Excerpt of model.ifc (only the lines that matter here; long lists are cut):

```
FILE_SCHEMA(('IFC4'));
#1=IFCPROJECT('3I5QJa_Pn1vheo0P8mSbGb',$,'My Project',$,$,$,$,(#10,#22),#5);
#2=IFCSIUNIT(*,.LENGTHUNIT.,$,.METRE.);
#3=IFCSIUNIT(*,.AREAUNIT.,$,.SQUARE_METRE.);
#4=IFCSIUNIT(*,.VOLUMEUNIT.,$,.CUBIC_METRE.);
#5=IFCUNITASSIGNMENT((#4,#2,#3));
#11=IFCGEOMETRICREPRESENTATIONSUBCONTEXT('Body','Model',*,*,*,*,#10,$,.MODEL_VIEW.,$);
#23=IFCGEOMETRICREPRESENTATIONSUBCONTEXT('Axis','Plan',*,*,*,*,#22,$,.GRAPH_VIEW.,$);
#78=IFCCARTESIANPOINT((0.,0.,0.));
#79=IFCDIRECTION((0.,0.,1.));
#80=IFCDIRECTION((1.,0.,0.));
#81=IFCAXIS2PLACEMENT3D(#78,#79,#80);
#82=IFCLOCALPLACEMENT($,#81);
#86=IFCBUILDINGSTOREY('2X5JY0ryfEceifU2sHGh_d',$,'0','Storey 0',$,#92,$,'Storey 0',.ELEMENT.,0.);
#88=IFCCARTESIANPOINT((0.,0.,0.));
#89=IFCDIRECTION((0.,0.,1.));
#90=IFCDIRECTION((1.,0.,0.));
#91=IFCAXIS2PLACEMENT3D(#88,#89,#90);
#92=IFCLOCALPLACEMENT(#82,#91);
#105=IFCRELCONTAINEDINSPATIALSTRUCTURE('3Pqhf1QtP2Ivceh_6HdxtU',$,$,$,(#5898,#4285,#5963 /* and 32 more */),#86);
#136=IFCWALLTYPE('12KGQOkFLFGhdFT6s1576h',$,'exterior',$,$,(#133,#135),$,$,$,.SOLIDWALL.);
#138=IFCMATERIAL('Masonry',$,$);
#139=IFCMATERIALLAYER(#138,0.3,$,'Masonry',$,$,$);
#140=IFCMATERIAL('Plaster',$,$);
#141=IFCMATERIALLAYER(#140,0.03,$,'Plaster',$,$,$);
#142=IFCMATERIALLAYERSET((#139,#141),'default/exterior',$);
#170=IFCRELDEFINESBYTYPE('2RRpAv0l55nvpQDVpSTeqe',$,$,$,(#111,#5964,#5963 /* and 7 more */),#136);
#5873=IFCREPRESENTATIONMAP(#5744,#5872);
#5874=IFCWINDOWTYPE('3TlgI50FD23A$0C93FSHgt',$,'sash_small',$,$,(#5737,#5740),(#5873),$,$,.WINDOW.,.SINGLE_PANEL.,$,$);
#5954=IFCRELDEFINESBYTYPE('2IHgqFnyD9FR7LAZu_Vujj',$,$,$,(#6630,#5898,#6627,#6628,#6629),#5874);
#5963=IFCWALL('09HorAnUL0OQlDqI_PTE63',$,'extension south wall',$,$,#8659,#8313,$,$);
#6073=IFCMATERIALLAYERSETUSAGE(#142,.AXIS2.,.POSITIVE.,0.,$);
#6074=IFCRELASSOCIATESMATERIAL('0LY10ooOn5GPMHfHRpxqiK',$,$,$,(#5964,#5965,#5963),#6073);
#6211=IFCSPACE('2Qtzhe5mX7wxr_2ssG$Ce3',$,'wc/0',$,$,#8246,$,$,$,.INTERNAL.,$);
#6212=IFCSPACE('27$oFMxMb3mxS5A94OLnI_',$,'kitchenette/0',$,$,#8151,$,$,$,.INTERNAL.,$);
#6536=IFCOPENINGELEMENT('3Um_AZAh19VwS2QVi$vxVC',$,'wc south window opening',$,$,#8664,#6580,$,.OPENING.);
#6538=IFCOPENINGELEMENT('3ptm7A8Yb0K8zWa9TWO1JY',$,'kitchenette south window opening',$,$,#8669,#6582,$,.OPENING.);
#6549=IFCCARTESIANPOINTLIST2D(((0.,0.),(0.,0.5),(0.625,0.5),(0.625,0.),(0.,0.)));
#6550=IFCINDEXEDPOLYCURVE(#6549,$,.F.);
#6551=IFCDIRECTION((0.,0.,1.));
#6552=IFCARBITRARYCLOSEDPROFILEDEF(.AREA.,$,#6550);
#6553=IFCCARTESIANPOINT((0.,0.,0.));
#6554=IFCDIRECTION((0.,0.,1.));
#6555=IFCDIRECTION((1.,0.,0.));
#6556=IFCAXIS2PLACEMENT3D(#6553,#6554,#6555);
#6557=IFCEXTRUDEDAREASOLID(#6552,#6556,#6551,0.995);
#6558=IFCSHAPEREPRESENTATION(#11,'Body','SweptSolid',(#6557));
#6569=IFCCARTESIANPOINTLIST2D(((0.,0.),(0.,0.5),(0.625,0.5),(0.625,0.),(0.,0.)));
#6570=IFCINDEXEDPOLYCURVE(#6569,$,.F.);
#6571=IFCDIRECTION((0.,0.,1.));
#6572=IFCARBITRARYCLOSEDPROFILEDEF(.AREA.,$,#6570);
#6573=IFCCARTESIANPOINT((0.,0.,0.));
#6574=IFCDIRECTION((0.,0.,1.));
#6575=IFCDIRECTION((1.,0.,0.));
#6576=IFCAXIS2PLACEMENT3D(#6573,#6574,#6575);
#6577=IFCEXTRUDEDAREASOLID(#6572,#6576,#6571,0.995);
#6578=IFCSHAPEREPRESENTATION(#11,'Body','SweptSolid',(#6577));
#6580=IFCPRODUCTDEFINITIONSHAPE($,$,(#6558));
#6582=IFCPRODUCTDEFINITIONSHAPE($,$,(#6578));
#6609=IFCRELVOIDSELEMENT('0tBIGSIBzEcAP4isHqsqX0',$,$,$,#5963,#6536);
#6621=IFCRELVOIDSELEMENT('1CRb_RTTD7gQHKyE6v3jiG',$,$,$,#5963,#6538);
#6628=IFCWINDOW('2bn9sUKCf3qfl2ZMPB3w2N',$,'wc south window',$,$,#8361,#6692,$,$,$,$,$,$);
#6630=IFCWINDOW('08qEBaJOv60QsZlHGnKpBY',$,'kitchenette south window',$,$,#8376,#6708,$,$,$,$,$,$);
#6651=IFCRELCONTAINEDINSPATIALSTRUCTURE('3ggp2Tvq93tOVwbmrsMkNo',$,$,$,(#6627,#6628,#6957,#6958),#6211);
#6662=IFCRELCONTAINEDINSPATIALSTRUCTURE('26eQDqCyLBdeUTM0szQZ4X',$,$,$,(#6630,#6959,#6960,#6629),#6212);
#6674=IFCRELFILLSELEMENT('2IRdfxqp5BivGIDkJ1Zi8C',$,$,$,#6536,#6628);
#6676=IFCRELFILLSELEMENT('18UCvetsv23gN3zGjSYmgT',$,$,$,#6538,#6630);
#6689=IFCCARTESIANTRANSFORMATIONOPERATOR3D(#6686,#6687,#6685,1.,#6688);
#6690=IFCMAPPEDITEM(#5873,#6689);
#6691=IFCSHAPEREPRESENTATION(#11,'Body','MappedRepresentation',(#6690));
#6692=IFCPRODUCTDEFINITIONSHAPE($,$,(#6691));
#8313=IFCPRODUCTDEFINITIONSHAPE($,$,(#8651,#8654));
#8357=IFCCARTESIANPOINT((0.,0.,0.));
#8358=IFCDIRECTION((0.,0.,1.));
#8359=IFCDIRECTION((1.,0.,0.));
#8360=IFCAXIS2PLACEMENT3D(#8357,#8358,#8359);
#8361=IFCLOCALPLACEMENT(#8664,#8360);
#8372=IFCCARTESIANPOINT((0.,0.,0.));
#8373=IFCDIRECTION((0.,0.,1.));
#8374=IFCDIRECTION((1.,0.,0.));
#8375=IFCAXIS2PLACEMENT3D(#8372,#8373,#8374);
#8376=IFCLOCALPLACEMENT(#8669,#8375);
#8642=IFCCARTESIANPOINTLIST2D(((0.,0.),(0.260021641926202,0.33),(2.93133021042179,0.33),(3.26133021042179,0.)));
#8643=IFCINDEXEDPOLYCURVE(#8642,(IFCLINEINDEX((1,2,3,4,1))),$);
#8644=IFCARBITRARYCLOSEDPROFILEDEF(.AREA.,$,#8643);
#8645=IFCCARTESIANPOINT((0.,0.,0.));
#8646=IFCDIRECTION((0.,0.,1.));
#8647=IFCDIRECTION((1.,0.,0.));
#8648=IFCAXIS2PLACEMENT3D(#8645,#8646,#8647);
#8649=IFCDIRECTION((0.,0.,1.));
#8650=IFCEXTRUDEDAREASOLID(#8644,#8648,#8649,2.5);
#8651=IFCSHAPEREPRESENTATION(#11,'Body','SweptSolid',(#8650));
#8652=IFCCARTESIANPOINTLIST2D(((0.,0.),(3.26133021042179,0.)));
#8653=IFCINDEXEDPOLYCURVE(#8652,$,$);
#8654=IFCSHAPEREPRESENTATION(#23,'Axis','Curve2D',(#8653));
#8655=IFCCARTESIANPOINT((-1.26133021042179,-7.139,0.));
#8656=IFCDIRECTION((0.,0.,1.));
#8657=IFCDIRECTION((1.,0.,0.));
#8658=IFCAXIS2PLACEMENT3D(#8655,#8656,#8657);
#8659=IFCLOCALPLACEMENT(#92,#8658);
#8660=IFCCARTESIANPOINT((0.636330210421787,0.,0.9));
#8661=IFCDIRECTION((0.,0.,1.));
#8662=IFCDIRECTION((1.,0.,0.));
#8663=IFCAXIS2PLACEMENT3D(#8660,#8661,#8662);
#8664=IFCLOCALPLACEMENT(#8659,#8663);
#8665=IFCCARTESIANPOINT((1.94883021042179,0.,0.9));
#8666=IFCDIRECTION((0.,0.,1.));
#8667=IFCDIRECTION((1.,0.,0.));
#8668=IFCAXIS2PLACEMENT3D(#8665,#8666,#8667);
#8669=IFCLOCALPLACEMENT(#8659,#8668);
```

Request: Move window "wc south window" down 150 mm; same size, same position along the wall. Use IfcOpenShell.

```python
import numpy as np
import ifcopenshell
import ifcopenshell.api.geometry
import ifcopenshell.util.placement
import ifcopenshell.util.unit

model = ifcopenshell.open("model.ifc")
unit_scale = ifcopenshell.util.unit.calculate_unit_scale(model)

window = model.by_guid("2bn9sUKCf3qfl2ZMPB3w2N")
opening = window.FillsVoids[0].RelatingOpeningElement
dz = -0.15 / unit_scale

shift = np.array([0.0, 0.0, dz])
# The window is placed relative to its opening, so it follows when the opening moves.
matrix = ifcopenshell.util.placement.get_local_placement(opening.ObjectPlacement)
matrix[:3, 3] += shift
ifcopenshell.api.geometry.edit_object_placement(
    model, product=opening, matrix=matrix, is_si=False, should_transform_children=True
)

print(f"moved by {dz * unit_scale:+.3f} m")

model.write("model_updated.ifc")
```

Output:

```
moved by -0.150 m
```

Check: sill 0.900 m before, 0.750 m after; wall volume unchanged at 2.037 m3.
